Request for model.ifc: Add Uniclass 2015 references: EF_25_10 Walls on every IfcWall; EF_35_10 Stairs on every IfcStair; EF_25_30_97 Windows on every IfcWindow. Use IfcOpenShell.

First a look at what the model holds.

```python
import ifcopenshell

model = ifcopenshell.open("model.ifc")
print(model.schema)
print("classifications:", [c.Name for c in model.by_type("IfcClassification")])
for ifc_class in ("IfcDoor", "IfcRoof", "IfcStair", "IfcWall", "IfcWindow"):
    print(ifc_class, len(model.by_type(ifc_class)))
```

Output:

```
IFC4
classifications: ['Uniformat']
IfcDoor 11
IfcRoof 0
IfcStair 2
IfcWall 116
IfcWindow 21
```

```python
import ifcopenshell
import ifcopenshell.api.classification

model = ifcopenshell.open("model.ifc")

system = ifcopenshell.api.classification.add_classification(model, classification="Uniclass 2015")

codes = {
    "IfcWall": ("EF_25_10", "Walls"),
    "IfcStair": ("EF_35_10", "Stairs"),
    "IfcWindow": ("EF_25_30_97", "Windows"),
}
for ifc_class, (code, name) in codes.items():
    products = model.by_type(ifc_class)
    ifcopenshell.api.classification.add_reference(
        model, products=products, classification=system, identification=code, name=name
    )
    print(code, len(products))

model.write("model_updated.ifc")
```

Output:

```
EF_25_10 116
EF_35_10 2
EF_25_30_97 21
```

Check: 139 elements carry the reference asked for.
